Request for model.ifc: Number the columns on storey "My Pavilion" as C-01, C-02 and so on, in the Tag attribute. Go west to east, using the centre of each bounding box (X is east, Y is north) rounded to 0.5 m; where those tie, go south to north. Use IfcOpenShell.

First a look at what the model holds.

```python
import ifcopenshell
import ifcopenshell.util.element
import ifcopenshell.util.placement

model = ifcopenshell.open("model.ifc")
print(model.schema)
storey = next(s for s in model.by_type("IfcBuildingStorey") if s.Name == "My Pavilion")
columns = [e for e in ifcopenshell.util.element.get_decomposition(storey) if e.is_a("IfcColumn")]
for e in sorted(columns, key=lambda e: e.id()):
    origin = ifcopenshell.util.placement.get_local_placement(e.ObjectPlacement)[:3, 3]
    print(e.id(), e.Tag, e.Name, origin.round(2) + 0.0, sep=" | ")
```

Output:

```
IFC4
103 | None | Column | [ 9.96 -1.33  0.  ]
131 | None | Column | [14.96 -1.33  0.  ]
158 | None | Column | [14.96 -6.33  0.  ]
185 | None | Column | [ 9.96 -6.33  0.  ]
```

```python
import ifcopenshell
import ifcopenshell.geom
import ifcopenshell.util.element
import ifcopenshell.util.shape

model = ifcopenshell.open("model.ifc")
settings = ifcopenshell.geom.settings()
settings.set("use-world-coords", True)


def centre(element):
    shape = ifcopenshell.geom.create_shape(settings, element)
    return ifcopenshell.util.shape.get_bbox_centroid(shape.geometry)


storey = next(s for s in model.by_type("IfcBuildingStorey") if s.Name == "My Pavilion")
columns = [e for e in ifcopenshell.util.element.get_decomposition(storey) if e.is_a("IfcColumn")]

# Insertion points can sit at a corner or the storey origin, so sort by the geometry (in metres).
centres = {e: centre(e) for e in columns}
columns.sort(key=lambda e: (round(centres[e][0] / 0.5), centres[e][1]))

for i, e in enumerate(columns, start=1):
    number = f"C-{i:02d}"
    e.Tag = number
    print(e.id(), number)

model.write("model_updated.ifc")
```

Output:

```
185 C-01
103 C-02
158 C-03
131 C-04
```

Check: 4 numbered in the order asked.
